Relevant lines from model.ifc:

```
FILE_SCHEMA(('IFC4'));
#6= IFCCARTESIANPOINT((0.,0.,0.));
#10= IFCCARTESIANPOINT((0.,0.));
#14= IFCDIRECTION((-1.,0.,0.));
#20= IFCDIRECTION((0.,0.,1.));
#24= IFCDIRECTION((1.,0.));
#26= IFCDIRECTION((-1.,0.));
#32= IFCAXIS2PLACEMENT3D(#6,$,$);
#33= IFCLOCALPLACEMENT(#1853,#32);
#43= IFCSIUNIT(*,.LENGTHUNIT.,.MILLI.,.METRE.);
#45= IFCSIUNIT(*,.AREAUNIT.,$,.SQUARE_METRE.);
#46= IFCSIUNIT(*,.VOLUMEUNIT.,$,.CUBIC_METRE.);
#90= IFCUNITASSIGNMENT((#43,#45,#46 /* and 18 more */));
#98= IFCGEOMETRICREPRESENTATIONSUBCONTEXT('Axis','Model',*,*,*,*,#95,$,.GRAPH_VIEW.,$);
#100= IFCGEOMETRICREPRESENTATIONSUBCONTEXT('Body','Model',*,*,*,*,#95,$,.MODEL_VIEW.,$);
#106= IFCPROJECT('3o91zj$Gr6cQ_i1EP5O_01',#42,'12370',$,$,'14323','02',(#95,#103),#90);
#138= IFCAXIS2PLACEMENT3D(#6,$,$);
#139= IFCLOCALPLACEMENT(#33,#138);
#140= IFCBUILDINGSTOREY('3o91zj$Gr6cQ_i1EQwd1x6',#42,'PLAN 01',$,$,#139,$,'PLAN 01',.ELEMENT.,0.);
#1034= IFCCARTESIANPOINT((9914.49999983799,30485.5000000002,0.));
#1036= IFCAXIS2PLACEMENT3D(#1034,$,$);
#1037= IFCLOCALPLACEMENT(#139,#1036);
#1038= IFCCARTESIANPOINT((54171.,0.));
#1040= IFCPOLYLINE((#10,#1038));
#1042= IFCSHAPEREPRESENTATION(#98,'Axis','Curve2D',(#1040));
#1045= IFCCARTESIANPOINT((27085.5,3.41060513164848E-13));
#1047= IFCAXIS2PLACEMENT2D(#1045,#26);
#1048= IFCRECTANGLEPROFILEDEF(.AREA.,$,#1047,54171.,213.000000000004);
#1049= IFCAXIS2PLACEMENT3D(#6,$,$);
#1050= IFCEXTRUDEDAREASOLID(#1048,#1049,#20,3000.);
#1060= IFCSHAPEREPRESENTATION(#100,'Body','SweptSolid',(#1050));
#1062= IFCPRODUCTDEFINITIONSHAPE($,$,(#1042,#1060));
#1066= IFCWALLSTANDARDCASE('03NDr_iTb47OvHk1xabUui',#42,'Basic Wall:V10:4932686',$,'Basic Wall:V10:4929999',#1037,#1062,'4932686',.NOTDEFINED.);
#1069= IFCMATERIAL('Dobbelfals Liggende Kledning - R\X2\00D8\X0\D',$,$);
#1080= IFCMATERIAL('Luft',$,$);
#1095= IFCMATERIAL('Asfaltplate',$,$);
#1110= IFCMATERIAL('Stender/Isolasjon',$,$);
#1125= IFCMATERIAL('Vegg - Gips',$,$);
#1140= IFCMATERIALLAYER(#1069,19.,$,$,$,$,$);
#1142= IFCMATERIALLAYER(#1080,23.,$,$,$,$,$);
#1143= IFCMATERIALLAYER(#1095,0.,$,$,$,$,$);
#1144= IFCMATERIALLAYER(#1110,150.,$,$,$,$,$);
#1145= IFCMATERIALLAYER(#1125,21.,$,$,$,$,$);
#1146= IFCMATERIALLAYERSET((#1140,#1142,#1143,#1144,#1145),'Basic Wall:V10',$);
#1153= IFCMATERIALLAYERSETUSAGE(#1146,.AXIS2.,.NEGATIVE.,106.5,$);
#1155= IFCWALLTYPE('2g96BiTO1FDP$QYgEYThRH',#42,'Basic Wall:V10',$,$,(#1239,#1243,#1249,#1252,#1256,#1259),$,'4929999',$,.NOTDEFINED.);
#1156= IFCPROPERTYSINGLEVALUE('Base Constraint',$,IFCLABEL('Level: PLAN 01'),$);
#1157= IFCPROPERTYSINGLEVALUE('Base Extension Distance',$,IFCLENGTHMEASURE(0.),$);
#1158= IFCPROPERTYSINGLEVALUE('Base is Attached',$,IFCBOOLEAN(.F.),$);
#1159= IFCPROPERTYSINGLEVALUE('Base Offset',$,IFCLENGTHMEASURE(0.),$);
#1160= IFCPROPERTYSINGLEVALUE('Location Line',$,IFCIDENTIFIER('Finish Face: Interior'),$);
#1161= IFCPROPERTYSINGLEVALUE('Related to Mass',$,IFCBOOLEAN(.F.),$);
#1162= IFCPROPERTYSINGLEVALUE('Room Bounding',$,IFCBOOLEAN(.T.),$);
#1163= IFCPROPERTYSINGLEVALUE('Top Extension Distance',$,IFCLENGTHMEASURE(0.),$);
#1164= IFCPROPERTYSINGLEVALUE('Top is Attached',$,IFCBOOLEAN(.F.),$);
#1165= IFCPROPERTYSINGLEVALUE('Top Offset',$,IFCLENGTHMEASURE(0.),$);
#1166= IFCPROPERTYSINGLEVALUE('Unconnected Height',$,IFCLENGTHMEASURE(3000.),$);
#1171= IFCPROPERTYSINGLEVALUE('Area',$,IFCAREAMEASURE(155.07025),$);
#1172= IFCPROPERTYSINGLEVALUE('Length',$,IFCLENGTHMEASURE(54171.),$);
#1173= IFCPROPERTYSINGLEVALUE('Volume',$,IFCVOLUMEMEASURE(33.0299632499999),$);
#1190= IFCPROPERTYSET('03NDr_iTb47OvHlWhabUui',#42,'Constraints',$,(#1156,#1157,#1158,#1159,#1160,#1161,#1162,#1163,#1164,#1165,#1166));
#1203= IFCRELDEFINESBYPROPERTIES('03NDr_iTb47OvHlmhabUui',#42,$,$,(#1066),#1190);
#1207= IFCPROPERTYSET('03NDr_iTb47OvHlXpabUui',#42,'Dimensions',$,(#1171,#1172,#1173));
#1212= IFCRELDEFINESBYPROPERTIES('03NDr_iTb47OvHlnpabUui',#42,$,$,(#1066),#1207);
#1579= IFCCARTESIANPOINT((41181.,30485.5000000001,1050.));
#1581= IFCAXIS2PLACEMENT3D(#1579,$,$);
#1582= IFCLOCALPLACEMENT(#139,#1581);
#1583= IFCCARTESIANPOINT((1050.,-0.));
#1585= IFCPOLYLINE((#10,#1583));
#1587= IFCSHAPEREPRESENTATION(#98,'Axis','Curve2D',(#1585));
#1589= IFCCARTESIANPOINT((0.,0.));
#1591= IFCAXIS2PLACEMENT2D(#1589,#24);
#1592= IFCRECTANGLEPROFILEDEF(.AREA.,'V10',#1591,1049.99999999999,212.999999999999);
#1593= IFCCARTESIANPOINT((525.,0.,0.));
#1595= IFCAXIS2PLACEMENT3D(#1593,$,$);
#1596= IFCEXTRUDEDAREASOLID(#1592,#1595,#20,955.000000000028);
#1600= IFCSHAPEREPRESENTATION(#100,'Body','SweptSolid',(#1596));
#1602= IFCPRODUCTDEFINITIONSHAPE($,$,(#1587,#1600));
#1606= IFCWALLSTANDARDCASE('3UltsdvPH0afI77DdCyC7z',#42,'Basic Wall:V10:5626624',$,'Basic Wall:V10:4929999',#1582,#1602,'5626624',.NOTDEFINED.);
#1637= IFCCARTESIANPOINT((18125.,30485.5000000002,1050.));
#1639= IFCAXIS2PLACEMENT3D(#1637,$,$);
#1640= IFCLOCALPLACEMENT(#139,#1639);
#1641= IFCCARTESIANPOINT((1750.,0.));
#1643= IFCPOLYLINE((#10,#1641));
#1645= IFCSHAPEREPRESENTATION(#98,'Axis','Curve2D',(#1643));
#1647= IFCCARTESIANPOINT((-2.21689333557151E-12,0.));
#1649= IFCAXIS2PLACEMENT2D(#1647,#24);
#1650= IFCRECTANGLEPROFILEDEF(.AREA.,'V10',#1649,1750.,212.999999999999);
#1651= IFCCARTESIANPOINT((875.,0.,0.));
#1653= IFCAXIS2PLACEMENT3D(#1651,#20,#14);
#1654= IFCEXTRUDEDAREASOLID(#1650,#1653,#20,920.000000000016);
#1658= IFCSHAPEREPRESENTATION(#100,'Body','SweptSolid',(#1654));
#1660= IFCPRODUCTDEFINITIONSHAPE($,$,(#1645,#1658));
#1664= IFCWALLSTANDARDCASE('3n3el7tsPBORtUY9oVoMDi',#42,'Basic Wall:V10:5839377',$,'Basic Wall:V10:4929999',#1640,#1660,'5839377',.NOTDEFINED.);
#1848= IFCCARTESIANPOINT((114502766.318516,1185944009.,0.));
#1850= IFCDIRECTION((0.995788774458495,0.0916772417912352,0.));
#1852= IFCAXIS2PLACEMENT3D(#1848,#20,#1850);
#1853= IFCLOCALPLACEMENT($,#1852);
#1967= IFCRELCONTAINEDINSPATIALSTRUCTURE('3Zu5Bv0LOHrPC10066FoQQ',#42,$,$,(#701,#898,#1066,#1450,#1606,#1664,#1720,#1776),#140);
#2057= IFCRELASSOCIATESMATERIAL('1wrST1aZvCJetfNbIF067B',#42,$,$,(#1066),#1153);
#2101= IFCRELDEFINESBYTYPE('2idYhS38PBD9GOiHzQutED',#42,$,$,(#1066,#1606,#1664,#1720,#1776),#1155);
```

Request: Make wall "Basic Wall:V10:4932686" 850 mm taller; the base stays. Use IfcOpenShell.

```python
import ifcopenshell
import ifcopenshell.api.pset
import ifcopenshell.geom
import ifcopenshell.util.element
import ifcopenshell.util.representation
import ifcopenshell.util.shape
import ifcopenshell.util.unit

model = ifcopenshell.open("model.ifc")
area_scale = ifcopenshell.util.unit.calculate_unit_scale(model, "AREAUNIT")
volume_scale = ifcopenshell.util.unit.calculate_unit_scale(model, "VOLUMEUNIT")
settings = ifcopenshell.geom.settings()


def volume(element):
    """Net volume in cubic metres, openings subtracted."""
    shape = ifcopenshell.geom.create_shape(settings, element)
    return ifcopenshell.util.shape.get_volume(shape.geometry)


wall = model.by_guid("03NDr_iTb47OvHk1xabUui")
before = volume(wall)

body = ifcopenshell.util.representation.get_representation(wall, "Model", "Body")
solid = body.Items[0]
old_height = solid.Depth
solid.Depth += 850.0
after = volume(wall)
thickness = 0.213  # wall thickness in metres

# Update the stored height, areas and volumes.
pset = model.by_id(ifcopenshell.util.element.get_pset(wall, "Constraints", should_inherit=False)["id"])
ifcopenshell.api.pset.edit_pset(model, pset=pset, properties={
    "Unconnected Height": model.create_entity("IfcLengthMeasure", solid.Depth),
})
pset = model.by_id(ifcopenshell.util.element.get_pset(wall, "Dimensions", should_inherit=False)["id"])
ifcopenshell.api.pset.edit_pset(model, pset=pset, properties={
    "Area": model.create_entity("IfcAreaMeasure", after / thickness / area_scale),
    "Volume": model.create_entity("IfcVolumeMeasure", after / volume_scale),
})

print(f"height {old_height:g} -> {solid.Depth:g}, volume {before:.3f} -> {after:.3f} m3")

model.write("model_edited.ifc")
```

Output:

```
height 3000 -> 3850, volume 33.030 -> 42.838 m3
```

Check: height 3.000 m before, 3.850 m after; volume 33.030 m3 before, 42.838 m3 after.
